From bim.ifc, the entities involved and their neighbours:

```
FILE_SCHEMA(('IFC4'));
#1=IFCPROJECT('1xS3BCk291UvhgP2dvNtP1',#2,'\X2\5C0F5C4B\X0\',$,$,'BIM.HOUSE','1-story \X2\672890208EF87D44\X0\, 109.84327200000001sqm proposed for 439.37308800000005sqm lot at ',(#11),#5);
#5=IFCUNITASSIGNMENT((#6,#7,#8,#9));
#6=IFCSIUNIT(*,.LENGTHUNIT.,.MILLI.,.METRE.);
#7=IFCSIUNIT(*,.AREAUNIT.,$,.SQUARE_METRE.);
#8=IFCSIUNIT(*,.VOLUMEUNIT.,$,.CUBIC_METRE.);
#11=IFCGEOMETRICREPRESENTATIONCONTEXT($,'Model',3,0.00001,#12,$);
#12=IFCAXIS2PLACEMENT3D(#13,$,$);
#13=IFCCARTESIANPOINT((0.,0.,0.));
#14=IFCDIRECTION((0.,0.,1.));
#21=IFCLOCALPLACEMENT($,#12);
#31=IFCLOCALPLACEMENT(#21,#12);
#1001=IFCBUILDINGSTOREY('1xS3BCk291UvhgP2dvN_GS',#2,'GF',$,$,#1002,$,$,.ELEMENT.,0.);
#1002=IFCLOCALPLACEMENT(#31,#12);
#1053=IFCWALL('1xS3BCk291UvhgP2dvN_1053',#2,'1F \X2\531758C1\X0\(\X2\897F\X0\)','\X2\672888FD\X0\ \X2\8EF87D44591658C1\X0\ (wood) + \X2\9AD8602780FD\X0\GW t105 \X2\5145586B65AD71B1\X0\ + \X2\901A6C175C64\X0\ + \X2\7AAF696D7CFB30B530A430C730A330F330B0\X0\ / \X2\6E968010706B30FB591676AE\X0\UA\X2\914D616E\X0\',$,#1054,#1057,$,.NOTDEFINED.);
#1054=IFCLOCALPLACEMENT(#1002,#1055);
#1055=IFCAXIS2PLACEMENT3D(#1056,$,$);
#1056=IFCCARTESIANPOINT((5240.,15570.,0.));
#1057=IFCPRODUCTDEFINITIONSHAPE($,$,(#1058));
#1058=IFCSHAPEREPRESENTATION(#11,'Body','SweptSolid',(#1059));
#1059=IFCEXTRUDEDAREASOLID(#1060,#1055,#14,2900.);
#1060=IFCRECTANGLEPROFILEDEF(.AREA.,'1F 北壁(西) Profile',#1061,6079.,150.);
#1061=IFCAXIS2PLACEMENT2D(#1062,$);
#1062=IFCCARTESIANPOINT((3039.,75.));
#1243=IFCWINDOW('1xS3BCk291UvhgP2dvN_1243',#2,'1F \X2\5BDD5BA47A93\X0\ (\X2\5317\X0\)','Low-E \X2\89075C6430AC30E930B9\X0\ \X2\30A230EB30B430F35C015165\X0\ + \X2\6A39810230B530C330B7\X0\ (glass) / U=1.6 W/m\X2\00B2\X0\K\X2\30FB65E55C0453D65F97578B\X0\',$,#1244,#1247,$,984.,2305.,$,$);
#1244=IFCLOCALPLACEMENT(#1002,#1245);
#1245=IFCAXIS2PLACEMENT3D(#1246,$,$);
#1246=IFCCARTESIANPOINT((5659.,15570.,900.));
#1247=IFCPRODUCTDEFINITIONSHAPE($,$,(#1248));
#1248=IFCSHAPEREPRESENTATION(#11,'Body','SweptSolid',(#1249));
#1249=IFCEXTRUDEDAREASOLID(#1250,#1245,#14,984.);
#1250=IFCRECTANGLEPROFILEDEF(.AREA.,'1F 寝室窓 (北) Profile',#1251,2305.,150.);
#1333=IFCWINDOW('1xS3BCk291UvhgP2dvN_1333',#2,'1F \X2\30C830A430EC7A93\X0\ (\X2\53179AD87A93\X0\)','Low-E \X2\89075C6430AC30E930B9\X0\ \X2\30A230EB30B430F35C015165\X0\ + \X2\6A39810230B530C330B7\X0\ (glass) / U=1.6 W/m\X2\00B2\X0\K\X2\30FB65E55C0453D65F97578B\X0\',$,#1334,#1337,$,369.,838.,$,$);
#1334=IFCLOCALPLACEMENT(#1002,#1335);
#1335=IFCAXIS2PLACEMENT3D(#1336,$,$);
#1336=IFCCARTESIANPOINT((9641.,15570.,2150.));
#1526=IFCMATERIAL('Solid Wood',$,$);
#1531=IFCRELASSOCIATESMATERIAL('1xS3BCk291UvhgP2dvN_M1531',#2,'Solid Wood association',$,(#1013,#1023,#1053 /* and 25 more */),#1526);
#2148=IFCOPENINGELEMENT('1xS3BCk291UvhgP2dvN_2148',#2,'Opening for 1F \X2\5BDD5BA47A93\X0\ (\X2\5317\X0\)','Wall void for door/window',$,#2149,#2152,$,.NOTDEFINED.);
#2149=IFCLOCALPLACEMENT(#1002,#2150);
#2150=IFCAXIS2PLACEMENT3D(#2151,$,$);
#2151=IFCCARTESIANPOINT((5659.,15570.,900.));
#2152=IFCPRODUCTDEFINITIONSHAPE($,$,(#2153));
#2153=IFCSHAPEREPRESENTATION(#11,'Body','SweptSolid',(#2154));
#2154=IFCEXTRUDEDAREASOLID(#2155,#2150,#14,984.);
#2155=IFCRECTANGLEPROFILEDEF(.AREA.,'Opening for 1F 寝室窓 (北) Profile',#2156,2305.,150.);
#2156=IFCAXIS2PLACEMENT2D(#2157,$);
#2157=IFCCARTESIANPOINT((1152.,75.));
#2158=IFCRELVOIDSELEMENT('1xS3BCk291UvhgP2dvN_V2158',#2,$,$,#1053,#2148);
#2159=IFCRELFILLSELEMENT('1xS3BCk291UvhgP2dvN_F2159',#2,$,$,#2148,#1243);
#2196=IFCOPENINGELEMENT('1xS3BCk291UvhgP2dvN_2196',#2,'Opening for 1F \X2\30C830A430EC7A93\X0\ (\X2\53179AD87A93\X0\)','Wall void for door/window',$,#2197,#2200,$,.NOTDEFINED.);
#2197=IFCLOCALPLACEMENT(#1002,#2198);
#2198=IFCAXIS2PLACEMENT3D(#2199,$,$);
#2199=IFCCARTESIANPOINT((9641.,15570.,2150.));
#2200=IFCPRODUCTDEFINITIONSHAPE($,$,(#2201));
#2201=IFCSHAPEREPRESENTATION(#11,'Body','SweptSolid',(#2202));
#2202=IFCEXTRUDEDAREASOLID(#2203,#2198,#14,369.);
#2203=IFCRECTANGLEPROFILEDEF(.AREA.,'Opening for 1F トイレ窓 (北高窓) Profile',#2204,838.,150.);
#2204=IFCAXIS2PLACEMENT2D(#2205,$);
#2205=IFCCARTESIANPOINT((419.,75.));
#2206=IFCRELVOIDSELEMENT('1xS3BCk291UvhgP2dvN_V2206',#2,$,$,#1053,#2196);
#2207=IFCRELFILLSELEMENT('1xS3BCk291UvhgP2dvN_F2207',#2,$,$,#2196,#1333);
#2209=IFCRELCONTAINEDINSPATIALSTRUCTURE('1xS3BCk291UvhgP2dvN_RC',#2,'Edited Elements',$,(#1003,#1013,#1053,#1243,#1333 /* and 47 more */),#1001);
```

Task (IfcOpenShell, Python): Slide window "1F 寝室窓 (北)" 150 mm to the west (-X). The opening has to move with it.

```python
import ifcopenshell
import ifcopenshell.api.geometry
import ifcopenshell.util.placement
import ifcopenshell.util.unit

model = ifcopenshell.open("bim.ifc")
unit_scale = ifcopenshell.util.unit.calculate_unit_scale(model)

window = model.by_guid("1xS3BCk291UvhgP2dvN_1243")
opening = window.FillsVoids[0].RelatingOpeningElement
wall = opening.VoidsElements[0].RelatingBuildingElement

wall_matrix = ifcopenshell.util.placement.get_local_placement(wall.ObjectPlacement)
shift = wall_matrix[:3, 0] * -0.15 / unit_scale
before = ifcopenshell.util.placement.get_local_placement(window.ObjectPlacement)[:3, 3].copy()

# The window is not placed relative to its opening, so move both.
for product in (opening, window):
    matrix = ifcopenshell.util.placement.get_local_placement(product.ObjectPlacement)
    matrix[:3, 3] += shift
    ifcopenshell.api.geometry.edit_object_placement(model, product=product, matrix=matrix, is_si=False)

after = ifcopenshell.util.placement.get_local_placement(window.ObjectPlacement)[:3, 3]
print("window moved by", (after - before).round(3) + 0.0)

model.write("bim_rev.ifc")
```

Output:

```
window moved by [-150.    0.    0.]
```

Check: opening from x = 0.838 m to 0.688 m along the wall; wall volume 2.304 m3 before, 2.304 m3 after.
